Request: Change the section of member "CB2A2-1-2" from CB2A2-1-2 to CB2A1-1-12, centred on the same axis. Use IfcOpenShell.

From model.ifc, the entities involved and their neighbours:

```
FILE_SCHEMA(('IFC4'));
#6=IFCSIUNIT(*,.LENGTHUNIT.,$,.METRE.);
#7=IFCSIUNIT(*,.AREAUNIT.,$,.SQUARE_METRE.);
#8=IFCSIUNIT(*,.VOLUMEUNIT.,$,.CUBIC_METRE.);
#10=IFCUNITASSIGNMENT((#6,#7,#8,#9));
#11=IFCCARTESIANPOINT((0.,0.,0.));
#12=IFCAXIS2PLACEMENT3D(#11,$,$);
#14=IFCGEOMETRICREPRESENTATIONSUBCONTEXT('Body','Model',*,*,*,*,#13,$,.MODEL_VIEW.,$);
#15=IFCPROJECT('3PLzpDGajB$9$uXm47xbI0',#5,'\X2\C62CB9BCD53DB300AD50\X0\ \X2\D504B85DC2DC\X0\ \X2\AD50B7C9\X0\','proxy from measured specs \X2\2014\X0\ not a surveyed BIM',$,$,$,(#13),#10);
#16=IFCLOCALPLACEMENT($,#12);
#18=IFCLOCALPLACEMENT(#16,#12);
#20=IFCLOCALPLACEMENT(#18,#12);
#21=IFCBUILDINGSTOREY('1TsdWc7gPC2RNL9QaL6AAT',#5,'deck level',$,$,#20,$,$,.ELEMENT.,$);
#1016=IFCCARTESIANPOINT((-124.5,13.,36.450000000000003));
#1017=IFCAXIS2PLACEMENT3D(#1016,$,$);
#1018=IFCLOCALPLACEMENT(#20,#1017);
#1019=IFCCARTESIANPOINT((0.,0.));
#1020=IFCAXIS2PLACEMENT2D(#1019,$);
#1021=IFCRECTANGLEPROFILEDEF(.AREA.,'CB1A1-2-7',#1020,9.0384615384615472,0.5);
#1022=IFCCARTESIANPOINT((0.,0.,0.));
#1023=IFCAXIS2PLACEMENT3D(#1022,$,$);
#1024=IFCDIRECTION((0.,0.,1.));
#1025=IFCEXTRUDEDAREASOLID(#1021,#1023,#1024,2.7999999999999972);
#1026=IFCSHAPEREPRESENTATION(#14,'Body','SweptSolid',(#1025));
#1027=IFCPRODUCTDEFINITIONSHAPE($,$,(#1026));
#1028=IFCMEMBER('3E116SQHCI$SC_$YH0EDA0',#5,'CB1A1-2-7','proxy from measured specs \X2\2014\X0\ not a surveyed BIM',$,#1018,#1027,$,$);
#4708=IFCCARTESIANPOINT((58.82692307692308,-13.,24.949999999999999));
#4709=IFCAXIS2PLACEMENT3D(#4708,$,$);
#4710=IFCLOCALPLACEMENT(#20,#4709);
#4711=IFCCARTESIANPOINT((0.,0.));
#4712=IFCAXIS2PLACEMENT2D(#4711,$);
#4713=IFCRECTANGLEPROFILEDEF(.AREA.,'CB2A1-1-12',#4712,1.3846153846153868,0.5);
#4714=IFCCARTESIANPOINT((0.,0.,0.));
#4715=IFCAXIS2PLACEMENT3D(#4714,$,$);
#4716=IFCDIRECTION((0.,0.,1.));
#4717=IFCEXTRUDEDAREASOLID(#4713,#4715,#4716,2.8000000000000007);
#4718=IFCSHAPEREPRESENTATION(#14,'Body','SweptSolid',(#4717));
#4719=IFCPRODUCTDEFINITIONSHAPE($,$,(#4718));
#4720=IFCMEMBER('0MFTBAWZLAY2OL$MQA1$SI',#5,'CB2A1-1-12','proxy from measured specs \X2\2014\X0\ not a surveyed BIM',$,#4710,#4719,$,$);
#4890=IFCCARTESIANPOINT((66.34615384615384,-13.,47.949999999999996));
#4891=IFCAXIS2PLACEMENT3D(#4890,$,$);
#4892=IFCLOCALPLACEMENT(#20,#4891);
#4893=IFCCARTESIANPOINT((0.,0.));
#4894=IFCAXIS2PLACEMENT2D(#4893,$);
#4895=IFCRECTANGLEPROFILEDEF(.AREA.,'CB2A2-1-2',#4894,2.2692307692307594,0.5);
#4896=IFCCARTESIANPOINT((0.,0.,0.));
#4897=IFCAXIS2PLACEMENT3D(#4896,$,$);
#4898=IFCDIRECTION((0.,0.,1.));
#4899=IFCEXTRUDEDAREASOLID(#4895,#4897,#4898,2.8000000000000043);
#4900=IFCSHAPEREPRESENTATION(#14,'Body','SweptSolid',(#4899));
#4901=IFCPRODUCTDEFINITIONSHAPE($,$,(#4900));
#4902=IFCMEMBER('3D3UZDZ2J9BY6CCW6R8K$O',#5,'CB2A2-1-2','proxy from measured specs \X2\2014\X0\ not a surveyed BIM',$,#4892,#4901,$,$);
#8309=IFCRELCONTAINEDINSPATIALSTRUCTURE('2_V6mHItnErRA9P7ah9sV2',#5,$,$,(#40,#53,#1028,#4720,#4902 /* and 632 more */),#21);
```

```python
import ifcopenshell
import ifcopenshell.util.element
import ifcopenshell.util.representation

model = ifcopenshell.open("model.ifc")

member = model.by_guid("3D3UZDZ2J9BY6CCW6R8K$O")
source = next(p for p in model.by_type("IfcRectangleProfileDef") if p.ProfileName == "CB2A1-1-12")

body = ifcopenshell.util.representation.get_representation(member, "Model", "Body")
solid = body.Items[0]
old_profile = solid.SweptArea

# Copy the section's sizes but keep this member's own profile position.
profile = ifcopenshell.util.element.copy(model, source)
profile.Position = old_profile.Position
solid.SweptArea = profile
if not model.get_total_inverses(old_profile):
    ifcopenshell.util.element.remove_deep2(model, old_profile)
member.Name = member.Name.replace("CB2A2-1-2", "CB2A1-1-12")

print(solid.SweptArea)

model.write("model-out.ifc")
```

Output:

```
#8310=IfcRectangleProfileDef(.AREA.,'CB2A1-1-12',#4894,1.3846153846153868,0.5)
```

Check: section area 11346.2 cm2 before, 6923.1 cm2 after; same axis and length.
